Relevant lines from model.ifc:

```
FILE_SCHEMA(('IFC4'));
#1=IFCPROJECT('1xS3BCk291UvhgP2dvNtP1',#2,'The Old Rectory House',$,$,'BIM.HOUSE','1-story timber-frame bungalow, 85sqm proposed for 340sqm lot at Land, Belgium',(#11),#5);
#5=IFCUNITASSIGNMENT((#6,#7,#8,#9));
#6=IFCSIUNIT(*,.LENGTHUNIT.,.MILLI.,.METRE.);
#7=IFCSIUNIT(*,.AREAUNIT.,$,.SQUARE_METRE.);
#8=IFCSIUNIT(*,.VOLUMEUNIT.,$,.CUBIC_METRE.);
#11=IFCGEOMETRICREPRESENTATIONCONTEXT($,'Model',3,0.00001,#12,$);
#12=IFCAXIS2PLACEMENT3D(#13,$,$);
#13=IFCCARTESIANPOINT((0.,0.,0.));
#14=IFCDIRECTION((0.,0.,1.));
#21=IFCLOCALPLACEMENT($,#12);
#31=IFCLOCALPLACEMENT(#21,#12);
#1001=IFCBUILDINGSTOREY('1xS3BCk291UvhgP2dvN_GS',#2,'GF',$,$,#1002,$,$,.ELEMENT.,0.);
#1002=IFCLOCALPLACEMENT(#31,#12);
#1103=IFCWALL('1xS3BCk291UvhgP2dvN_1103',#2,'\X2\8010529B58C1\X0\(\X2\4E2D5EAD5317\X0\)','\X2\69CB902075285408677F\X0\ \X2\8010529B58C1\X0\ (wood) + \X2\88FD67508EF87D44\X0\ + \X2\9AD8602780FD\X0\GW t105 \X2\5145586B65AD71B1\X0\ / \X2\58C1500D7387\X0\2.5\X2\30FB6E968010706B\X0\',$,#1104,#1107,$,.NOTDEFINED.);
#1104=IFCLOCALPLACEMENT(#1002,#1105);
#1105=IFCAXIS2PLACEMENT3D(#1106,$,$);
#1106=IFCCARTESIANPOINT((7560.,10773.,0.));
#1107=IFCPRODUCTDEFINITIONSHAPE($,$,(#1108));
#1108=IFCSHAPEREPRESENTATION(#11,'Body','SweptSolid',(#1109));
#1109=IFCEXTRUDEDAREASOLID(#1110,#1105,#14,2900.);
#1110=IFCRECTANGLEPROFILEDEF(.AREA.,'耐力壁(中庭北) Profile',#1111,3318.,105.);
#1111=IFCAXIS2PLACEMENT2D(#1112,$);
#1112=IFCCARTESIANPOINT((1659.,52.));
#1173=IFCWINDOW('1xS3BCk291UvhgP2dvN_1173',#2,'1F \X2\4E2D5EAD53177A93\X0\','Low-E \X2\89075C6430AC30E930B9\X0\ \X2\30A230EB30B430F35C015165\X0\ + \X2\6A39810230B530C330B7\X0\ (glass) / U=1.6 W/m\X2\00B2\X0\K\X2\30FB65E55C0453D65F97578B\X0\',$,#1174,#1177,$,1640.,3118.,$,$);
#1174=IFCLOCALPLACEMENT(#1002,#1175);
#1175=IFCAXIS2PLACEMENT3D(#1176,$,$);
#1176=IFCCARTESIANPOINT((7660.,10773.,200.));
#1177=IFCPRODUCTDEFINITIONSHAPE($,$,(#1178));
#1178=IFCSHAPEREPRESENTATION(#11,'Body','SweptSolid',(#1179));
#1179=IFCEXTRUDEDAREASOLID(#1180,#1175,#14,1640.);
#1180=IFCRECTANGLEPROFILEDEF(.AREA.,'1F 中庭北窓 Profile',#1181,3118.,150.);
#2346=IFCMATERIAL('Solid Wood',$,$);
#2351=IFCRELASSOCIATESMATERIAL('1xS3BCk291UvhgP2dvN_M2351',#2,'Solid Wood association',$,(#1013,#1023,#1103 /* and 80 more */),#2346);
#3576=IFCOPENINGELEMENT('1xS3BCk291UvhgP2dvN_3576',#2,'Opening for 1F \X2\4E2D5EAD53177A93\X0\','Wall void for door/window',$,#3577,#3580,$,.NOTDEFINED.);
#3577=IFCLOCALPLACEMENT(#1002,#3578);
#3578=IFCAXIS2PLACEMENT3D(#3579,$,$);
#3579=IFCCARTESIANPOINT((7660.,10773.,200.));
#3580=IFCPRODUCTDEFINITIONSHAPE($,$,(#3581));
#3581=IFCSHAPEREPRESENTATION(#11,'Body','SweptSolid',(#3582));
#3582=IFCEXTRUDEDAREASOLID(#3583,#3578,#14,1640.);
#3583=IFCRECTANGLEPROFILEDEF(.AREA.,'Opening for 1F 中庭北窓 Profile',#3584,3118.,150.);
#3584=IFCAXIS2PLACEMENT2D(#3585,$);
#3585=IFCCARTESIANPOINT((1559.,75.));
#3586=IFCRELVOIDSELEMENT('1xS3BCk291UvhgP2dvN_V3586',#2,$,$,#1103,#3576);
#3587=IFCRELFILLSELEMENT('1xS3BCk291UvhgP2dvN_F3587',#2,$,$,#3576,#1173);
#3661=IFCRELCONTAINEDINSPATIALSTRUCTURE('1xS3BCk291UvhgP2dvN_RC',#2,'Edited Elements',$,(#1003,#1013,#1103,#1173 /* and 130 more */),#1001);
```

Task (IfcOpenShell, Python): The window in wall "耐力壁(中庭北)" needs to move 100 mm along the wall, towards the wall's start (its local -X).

```python
import ifcopenshell
import ifcopenshell.api.geometry
import ifcopenshell.util.placement
import ifcopenshell.util.unit

model = ifcopenshell.open("model.ifc")
unit_scale = ifcopenshell.util.unit.calculate_unit_scale(model)

window = model.by_id(1173)
opening = window.FillsVoids[0].RelatingOpeningElement
wall = opening.VoidsElements[0].RelatingBuildingElement

wall_matrix = ifcopenshell.util.placement.get_local_placement(wall.ObjectPlacement)
shift = wall_matrix[:3, 0] * -0.1 / unit_scale
before = ifcopenshell.util.placement.get_local_placement(window.ObjectPlacement)[:3, 3].copy()

# The window is not placed relative to its opening, so move both.
for product in (opening, window):
    matrix = ifcopenshell.util.placement.get_local_placement(product.ObjectPlacement)
    matrix[:3, 3] += shift
    ifcopenshell.api.geometry.edit_object_placement(model, product=product, matrix=matrix, is_si=False)

after = ifcopenshell.util.placement.get_local_placement(window.ObjectPlacement)[:3, 3]
print("window moved by", (after - before).round(3) + 0.0)

model.write("model_updated.ifc")
```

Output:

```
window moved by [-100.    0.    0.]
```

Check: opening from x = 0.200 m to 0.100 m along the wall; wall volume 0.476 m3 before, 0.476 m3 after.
